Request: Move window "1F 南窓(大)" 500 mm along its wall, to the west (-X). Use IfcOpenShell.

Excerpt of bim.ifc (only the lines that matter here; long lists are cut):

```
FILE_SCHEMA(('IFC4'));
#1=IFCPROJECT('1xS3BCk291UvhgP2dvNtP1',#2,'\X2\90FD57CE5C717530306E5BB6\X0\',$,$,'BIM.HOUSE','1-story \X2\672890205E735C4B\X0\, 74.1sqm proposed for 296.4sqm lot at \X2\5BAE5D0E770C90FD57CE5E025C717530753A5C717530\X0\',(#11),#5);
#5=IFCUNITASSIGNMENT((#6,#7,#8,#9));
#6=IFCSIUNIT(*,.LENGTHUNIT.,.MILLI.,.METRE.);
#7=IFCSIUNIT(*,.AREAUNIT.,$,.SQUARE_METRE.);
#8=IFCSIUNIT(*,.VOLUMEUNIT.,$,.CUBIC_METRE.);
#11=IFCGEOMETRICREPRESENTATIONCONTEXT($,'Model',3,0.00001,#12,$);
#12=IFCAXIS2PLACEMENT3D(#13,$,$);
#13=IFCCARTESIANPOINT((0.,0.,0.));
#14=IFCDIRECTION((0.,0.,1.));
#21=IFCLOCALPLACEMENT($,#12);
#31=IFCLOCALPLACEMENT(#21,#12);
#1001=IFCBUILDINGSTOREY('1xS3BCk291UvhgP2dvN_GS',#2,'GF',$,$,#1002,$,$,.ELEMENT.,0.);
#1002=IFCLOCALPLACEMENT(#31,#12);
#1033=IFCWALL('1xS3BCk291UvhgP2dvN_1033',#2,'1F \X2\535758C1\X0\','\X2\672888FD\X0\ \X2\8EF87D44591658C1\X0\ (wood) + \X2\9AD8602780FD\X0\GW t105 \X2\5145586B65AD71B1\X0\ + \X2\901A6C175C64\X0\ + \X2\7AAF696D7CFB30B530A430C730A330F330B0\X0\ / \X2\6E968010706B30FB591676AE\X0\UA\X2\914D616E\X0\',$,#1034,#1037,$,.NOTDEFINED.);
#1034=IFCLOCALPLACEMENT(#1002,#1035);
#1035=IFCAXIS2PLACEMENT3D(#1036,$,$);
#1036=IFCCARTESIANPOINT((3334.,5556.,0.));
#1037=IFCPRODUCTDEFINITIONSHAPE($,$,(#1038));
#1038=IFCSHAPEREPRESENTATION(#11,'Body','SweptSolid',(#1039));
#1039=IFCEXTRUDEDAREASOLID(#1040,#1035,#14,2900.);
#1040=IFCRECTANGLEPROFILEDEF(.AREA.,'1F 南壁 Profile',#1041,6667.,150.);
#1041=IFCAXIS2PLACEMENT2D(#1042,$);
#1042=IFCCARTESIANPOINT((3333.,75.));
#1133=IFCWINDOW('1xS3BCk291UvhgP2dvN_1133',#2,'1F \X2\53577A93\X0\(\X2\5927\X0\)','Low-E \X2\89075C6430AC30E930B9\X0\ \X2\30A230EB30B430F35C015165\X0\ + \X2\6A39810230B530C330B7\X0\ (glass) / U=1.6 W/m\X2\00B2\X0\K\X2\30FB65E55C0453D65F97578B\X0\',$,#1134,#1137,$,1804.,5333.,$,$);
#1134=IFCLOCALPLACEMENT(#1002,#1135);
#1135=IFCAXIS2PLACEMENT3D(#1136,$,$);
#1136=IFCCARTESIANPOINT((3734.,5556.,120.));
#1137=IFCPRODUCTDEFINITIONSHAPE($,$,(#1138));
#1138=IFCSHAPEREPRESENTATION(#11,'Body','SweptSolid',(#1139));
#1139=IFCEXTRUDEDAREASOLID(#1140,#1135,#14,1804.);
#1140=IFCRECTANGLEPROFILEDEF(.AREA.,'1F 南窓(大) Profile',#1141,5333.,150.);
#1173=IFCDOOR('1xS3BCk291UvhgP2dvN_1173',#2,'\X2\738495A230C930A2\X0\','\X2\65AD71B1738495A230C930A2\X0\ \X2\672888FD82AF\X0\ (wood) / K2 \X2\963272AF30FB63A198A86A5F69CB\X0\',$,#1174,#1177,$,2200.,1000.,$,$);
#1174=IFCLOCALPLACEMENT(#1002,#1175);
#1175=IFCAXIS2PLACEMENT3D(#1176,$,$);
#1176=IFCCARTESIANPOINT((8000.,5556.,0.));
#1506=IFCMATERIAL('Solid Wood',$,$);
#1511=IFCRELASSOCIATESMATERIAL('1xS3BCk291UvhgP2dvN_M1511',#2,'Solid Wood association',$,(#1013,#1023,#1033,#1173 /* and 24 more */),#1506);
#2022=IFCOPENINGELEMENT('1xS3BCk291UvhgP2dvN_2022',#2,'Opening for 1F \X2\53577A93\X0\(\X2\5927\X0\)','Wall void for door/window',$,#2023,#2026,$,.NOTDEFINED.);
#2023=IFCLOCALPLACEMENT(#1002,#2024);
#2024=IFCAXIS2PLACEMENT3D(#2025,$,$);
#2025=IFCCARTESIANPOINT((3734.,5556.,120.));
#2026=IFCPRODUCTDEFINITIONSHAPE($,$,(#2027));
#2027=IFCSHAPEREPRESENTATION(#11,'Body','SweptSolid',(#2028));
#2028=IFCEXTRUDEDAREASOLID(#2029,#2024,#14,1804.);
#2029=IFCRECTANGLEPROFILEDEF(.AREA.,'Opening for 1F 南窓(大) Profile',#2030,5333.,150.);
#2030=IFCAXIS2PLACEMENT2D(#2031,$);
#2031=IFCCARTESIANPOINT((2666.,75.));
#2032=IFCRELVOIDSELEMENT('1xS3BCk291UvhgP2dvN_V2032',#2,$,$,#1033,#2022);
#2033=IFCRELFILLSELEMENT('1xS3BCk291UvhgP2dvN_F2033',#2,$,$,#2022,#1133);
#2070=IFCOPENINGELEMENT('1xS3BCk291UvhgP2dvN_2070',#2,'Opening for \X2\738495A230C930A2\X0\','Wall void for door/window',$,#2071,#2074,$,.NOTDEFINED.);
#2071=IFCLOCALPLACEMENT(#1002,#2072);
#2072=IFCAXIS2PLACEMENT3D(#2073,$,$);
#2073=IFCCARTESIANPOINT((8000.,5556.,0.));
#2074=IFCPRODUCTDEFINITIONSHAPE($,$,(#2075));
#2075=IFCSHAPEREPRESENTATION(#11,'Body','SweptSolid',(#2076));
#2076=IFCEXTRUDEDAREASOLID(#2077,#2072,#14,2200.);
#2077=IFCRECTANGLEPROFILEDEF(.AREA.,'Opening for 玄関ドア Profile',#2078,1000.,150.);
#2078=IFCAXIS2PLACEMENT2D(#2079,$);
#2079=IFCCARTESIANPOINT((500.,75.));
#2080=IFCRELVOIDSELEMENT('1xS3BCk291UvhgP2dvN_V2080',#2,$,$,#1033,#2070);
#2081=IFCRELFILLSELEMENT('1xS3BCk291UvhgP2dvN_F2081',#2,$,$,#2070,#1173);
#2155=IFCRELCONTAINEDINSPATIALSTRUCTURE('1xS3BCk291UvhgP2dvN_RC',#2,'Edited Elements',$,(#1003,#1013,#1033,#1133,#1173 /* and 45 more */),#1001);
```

```python
import ifcopenshell
import ifcopenshell.api.geometry
import ifcopenshell.util.placement

model = ifcopenshell.open("bim.ifc")

window = model.by_guid("1xS3BCk291UvhgP2dvN_1133")
opening = window.FillsVoids[0].RelatingOpeningElement
wall = opening.VoidsElements[0].RelatingBuildingElement

wall_matrix = ifcopenshell.util.placement.get_local_placement(wall.ObjectPlacement)
shift = wall_matrix[:3, 0] * -500.0
before = ifcopenshell.util.placement.get_local_placement(window.ObjectPlacement)[:3, 3].copy()

# The window is not placed relative to its opening, so move both.
for product in (opening, window):
    matrix = ifcopenshell.util.placement.get_local_placement(product.ObjectPlacement)
    matrix[:3, 3] += shift
    ifcopenshell.api.geometry.edit_object_placement(model, product=product, matrix=matrix, is_si=False)

after = ifcopenshell.util.placement.get_local_placement(window.ObjectPlacement)[:3, 3]
print("window moved by", (after - before).round(3) + 0.0)

model.write("bim-out.ifc")
```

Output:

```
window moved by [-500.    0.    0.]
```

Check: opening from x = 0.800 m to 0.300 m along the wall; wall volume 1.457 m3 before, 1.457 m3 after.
